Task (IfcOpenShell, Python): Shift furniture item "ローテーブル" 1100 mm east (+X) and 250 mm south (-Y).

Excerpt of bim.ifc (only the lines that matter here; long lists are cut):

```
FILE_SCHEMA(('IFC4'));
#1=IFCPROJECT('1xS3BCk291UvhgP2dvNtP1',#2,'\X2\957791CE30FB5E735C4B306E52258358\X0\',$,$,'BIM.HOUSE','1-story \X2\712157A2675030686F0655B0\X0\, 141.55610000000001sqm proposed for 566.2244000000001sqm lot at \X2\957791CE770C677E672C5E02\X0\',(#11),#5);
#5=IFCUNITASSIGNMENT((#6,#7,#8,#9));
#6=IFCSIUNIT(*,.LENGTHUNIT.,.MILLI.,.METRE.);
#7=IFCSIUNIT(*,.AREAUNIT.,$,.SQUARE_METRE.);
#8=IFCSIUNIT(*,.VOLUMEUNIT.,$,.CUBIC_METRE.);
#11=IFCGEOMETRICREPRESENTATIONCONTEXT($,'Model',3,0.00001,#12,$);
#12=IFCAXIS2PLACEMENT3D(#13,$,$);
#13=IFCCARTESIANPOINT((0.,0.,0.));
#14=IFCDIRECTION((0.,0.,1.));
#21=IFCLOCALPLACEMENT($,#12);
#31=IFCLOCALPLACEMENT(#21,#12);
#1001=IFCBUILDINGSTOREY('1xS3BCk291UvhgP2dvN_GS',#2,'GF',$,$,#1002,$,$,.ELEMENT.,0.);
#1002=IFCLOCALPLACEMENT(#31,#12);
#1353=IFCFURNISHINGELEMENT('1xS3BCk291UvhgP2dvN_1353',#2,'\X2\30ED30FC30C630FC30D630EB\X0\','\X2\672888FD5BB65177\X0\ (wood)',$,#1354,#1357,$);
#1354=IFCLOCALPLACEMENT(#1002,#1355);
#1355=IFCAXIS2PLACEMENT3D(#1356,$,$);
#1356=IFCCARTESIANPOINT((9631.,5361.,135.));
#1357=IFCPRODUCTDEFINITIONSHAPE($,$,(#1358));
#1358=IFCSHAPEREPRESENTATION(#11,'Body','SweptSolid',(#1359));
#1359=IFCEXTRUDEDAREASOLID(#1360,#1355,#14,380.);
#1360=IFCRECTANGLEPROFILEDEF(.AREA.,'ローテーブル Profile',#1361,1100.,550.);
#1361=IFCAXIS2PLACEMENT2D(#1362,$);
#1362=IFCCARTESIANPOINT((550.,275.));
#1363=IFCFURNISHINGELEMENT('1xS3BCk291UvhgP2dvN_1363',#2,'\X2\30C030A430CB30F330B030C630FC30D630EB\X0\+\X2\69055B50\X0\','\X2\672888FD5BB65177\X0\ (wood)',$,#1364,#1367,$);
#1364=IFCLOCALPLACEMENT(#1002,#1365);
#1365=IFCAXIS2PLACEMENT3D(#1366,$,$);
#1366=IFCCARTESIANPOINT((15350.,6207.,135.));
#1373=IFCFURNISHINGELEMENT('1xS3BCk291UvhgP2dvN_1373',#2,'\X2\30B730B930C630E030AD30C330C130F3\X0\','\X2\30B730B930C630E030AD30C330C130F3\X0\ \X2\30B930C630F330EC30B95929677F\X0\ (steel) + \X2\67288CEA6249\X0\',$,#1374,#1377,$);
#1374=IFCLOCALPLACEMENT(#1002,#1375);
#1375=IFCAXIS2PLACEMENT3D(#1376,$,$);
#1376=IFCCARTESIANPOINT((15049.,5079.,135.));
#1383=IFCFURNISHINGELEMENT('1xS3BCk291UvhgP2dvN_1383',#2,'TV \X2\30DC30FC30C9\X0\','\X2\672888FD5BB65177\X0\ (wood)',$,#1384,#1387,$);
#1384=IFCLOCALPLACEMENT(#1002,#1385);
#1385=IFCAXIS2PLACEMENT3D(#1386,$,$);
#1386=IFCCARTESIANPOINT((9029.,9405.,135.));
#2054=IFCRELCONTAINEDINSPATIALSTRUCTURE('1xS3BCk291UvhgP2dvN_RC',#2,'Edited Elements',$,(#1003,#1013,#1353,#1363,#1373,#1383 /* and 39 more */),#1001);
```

```python
import ifcopenshell
import ifcopenshell.api.geometry
import ifcopenshell.util.placement
import ifcopenshell.util.unit

model = ifcopenshell.open("bim.ifc")
unit_scale = ifcopenshell.util.unit.calculate_unit_scale(model)

item = model.by_guid("1xS3BCk291UvhgP2dvN_1353")
matrix = ifcopenshell.util.placement.get_local_placement(item.ObjectPlacement)
matrix[0, 3] += 1.1 / unit_scale
matrix[1, 3] -= 0.25 / unit_scale
ifcopenshell.api.geometry.edit_object_placement(model, product=item, matrix=matrix, is_si=False)

print(ifcopenshell.util.placement.get_local_placement(item.ObjectPlacement).round(3) + 0.0)

model.write("bim_edited.ifc")
```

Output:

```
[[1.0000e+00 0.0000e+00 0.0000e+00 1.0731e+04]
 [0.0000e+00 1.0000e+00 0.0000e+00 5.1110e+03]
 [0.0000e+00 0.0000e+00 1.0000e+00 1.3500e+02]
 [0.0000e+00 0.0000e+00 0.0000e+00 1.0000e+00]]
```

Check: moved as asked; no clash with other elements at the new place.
